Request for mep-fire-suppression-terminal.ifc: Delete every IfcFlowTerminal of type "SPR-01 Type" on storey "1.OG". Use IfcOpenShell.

First a look at what the model holds.

```python
import ifcopenshell
import ifcopenshell.util.element

model = ifcopenshell.open("mep-fire-suppression-terminal.ifc")
print(model.schema)
storey = next(s for s in model.by_type("IfcBuildingStorey") if s.Name == "1.OG")
terminals = [e for e in ifcopenshell.util.element.get_decomposition(storey) if e.is_a("IfcFlowTerminal")]
seen = {}
for e in terminals:
    element_type = ifcopenshell.util.element.get_type(e)
    name = element_type.Name if element_type not in (None, e) else None
    seen[name] = seen.get(name, 0) + 1
for name, count in sorted(seen.items(), key=str):
    print(count, "x", name)
```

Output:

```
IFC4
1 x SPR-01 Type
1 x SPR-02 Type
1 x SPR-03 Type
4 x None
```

```python
import ifcopenshell
import ifcopenshell.api.root
import ifcopenshell.util.element

model = ifcopenshell.open("mep-fire-suppression-terminal.ifc")

storey = next(s for s in model.by_type("IfcBuildingStorey") if s.Name == "1.OG")
terminals = [e for e in ifcopenshell.util.element.get_decomposition(storey) if e.is_a("IfcFlowTerminal")]
targets = [e for e in terminals if (t := ifcopenshell.util.element.get_type(e)) not in (None, e) and t.Name == "SPR-01 Type"]

for e in targets:
    ifcopenshell.api.root.remove_product(model, product=e)
print(len(targets), "removed")

model.write("mep-fire-suppression-terminal-out.ifc")
```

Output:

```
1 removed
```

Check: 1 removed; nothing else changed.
